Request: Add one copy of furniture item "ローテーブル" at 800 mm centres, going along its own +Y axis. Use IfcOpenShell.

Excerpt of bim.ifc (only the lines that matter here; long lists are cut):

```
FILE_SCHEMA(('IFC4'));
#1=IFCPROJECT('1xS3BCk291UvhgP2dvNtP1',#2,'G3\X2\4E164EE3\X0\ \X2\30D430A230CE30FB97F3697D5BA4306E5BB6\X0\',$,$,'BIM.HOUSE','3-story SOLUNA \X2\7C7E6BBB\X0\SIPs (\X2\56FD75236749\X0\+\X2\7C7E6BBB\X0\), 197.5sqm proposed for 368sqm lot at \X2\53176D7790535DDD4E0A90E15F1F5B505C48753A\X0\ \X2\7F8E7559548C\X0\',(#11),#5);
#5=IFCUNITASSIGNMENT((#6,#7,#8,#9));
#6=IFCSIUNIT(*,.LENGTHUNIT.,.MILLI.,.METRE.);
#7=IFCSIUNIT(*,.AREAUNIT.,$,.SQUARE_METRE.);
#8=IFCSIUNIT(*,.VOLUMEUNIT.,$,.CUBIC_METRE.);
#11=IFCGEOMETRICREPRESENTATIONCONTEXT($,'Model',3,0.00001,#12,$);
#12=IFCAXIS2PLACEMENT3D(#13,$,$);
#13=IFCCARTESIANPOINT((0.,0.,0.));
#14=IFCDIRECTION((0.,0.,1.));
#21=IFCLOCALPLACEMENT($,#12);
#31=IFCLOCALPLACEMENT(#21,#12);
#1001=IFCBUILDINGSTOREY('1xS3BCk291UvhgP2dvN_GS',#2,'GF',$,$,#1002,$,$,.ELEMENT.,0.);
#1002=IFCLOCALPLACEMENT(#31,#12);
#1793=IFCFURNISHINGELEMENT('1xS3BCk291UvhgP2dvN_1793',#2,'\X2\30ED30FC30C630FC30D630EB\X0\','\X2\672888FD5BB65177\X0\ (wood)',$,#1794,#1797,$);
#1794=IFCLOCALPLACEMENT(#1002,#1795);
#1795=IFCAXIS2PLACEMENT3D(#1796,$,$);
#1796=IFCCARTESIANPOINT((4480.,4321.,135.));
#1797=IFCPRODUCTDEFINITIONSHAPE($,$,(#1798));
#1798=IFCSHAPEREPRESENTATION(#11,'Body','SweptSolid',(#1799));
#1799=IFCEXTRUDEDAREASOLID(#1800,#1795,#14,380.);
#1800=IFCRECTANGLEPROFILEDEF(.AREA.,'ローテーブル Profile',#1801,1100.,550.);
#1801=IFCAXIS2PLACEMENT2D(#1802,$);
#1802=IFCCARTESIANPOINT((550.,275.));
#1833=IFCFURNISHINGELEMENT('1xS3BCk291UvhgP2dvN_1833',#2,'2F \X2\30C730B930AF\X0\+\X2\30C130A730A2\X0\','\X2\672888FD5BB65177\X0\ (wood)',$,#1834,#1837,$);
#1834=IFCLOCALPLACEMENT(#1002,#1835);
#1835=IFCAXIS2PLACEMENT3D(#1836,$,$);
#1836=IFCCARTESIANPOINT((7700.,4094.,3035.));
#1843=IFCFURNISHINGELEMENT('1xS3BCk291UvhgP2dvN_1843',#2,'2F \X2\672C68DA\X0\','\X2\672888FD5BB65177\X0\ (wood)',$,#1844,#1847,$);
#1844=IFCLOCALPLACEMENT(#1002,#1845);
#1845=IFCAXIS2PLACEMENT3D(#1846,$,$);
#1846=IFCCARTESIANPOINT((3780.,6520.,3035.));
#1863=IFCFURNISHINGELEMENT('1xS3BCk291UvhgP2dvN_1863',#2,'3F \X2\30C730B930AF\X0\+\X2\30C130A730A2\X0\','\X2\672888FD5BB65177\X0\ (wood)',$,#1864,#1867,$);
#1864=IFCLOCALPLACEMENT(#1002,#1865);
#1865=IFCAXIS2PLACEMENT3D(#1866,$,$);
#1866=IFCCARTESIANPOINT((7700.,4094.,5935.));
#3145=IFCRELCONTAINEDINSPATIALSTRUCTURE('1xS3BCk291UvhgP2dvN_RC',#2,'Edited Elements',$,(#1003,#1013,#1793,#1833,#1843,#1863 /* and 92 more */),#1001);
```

```python
import ifcopenshell
import ifcopenshell.api.geometry
import ifcopenshell.api.root
import ifcopenshell.util.element
import ifcopenshell.util.placement
import ifcopenshell.util.unit

model = ifcopenshell.open("bim.ifc")
unit_scale = ifcopenshell.util.unit.calculate_unit_scale(model)


def reuse_history(source, copy):
    """copy_class also copies each property set's owner history, people and application; keep the originals."""
    for rel in copy.IsDefinedBy:
        if rel.is_a("IfcRelDefinesByProperties") and (history := rel.RelatingPropertyDefinition.OwnerHistory):
            rel.RelatingPropertyDefinition.OwnerHistory = source.OwnerHistory
            ifcopenshell.util.element.remove_deep2(model, history)


source = model.by_id(1793)
base = ifcopenshell.util.placement.get_local_placement(source.ObjectPlacement)
step = base[:3, 1] * 0.8 / unit_scale

for i in range(1, 2):
    copy = ifcopenshell.api.root.copy_class(model, product=source)
    copy.Representation = ifcopenshell.util.element.copy_deep(
        model, source.Representation, exclude=["IfcGeometricRepresentationContext", "IfcRepresentationMap"]
    )
    reuse_history(source, copy)
    matrix = base.copy()
    matrix[:3, 3] += i * step
    print("added at", matrix[:3, 3].round(3) + 0.0)
    ifcopenshell.api.geometry.edit_object_placement(model, product=copy, matrix=matrix, is_si=False)

model.write("bim_rev.ifc")
```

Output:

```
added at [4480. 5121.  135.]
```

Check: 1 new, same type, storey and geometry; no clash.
